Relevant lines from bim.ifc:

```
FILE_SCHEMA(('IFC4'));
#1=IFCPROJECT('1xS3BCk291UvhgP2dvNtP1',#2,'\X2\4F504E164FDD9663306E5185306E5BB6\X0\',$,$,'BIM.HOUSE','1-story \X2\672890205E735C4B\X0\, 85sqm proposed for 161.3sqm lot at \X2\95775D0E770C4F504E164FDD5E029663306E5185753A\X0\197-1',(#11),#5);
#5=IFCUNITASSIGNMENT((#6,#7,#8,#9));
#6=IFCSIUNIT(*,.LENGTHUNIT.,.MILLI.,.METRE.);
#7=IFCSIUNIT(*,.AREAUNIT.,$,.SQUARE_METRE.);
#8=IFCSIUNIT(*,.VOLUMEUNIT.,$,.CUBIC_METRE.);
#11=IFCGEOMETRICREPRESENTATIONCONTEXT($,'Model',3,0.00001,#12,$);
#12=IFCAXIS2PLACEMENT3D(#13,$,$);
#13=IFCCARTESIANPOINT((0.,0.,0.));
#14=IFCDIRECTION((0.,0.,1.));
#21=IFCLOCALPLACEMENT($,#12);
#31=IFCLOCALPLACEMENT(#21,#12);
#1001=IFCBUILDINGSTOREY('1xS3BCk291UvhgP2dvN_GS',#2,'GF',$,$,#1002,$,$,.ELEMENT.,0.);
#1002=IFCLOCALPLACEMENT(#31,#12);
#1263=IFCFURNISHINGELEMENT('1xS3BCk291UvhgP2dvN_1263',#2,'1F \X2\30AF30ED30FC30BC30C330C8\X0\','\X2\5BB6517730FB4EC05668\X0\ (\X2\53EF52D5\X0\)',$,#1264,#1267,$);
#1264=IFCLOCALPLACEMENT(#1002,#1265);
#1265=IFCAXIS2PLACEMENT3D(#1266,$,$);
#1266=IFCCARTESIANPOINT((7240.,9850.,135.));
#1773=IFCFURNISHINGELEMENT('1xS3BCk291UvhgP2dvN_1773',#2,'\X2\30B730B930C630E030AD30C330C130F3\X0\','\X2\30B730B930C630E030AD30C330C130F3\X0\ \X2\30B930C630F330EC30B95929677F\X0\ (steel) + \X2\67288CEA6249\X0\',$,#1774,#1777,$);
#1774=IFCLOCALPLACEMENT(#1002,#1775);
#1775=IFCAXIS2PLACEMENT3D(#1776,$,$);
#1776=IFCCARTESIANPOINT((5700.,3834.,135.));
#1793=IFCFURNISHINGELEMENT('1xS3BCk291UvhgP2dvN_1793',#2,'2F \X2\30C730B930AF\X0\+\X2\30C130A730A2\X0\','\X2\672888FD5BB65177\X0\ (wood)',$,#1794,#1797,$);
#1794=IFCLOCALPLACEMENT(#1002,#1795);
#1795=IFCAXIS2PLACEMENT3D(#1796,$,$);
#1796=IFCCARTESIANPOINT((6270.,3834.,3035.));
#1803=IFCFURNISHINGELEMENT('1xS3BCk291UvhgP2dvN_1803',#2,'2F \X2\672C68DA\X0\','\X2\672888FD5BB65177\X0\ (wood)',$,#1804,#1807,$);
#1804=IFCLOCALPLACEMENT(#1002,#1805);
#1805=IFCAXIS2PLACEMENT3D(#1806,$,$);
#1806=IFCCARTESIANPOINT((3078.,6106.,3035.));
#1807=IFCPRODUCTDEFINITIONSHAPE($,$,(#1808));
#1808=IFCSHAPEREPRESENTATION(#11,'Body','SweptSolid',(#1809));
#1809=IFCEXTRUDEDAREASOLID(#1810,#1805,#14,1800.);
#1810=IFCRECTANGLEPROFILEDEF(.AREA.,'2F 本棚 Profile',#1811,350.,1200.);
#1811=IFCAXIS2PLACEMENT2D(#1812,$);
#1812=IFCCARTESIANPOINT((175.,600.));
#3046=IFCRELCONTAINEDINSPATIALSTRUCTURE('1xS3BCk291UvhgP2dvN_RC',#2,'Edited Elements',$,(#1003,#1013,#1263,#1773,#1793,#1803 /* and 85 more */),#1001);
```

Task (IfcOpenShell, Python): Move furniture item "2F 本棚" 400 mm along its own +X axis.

```python
import ifcopenshell
import ifcopenshell.api.geometry
import ifcopenshell.util.placement
import ifcopenshell.util.unit

model = ifcopenshell.open("bim.ifc")
unit_scale = ifcopenshell.util.unit.calculate_unit_scale(model)

item = model.by_guid("1xS3BCk291UvhgP2dvN_1803")
matrix = ifcopenshell.util.placement.get_local_placement(item.ObjectPlacement)
matrix[:3, 3] += matrix[:3, 0] * 0.4 / unit_scale
ifcopenshell.api.geometry.edit_object_placement(model, product=item, matrix=matrix, is_si=False)

print(ifcopenshell.util.placement.get_local_placement(item.ObjectPlacement).round(3) + 0.0)

model.write("bim_v2.ifc")
```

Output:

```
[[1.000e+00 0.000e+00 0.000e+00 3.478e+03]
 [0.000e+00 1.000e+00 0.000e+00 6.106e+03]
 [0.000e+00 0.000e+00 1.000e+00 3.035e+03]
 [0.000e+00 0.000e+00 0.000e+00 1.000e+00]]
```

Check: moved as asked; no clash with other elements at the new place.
